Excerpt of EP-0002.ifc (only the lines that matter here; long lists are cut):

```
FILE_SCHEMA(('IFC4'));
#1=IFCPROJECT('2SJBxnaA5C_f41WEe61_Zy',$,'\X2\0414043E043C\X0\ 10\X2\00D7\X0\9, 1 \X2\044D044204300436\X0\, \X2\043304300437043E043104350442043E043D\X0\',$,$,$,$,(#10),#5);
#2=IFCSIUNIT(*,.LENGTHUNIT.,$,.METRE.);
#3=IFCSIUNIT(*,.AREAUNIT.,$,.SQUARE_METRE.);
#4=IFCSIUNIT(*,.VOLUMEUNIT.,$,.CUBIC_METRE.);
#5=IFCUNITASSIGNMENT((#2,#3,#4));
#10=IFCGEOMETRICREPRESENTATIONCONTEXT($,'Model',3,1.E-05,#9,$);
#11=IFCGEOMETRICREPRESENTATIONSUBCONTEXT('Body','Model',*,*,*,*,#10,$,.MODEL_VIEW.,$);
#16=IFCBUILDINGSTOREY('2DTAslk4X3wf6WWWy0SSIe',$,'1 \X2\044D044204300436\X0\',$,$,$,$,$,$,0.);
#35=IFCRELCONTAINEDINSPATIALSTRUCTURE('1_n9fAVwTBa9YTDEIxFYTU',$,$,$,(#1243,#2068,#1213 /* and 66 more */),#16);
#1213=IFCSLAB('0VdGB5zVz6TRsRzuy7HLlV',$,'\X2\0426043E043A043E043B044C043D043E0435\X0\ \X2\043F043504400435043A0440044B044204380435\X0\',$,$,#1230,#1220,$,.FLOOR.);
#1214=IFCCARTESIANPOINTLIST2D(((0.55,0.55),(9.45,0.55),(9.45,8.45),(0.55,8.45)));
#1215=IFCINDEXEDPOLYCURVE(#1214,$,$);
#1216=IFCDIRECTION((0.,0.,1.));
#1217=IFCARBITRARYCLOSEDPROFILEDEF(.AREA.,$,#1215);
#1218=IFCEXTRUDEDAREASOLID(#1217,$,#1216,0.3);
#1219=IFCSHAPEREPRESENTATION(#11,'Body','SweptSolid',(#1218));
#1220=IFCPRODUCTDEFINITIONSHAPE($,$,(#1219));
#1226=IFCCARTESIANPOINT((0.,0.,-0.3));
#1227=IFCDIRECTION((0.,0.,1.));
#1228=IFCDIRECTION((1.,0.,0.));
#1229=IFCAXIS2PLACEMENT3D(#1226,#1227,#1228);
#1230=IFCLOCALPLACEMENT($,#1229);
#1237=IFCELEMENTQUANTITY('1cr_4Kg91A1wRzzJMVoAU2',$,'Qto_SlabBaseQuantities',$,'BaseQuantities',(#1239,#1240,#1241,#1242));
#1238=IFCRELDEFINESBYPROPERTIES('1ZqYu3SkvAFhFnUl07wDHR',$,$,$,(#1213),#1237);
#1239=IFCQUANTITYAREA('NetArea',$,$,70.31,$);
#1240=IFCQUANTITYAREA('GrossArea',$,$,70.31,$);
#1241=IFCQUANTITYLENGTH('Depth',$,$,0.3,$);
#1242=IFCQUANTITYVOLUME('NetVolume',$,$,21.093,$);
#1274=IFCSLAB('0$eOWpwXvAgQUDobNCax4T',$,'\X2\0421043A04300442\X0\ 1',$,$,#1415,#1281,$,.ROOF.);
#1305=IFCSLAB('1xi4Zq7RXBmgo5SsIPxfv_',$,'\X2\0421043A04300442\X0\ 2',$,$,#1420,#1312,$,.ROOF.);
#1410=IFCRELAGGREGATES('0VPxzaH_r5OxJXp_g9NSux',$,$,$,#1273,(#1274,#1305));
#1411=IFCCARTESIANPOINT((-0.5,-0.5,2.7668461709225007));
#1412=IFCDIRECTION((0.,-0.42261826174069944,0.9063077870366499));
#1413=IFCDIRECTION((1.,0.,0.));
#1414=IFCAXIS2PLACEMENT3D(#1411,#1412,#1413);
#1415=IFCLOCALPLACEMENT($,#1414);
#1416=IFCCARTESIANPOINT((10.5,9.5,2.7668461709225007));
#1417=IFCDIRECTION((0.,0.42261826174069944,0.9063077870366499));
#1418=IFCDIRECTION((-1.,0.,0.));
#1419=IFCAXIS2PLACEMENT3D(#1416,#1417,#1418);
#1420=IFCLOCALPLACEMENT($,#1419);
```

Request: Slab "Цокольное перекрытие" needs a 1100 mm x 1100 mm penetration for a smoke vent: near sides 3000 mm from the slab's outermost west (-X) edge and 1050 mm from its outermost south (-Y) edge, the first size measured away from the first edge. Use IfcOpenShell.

```python
import numpy as np
import ifcopenshell
import ifcopenshell.api.feature
import ifcopenshell.api.geometry
import ifcopenshell.api.pset
import ifcopenshell.api.root
import ifcopenshell.geom
import ifcopenshell.util.element
import ifcopenshell.util.placement
import ifcopenshell.util.representation
import ifcopenshell.util.shape
import ifcopenshell.util.unit

model = ifcopenshell.open("EP-0002.ifc")
unit_scale = ifcopenshell.util.unit.calculate_unit_scale(model)
area_scale = ifcopenshell.util.unit.calculate_unit_scale(model, "AREAUNIT")
volume_scale = ifcopenshell.util.unit.calculate_unit_scale(model, "VOLUMEUNIT")
settings = ifcopenshell.geom.settings()


def volume(element):
    """Net volume in cubic metres, openings subtracted."""
    shape = ifcopenshell.geom.create_shape(settings, element)
    return ifcopenshell.util.shape.get_volume(shape.geometry)


slab = model.by_guid("0VdGB5zVz6TRsRzuy7HLlV")
before = volume(slab)

# Extent in the slab's own axes, in metres. The edges named are its -X and -Y sides.
slab_shape = ifcopenshell.geom.create_shape(settings, slab)
vertices = ifcopenshell.util.shape.get_vertices(slab_shape.geometry)
x_min, y_min, bottom = vertices.min(axis=0)
top = vertices[:, 2].max()

opening = ifcopenshell.api.root.create_entity(model, ifc_class="IfcOpeningElement", name="Smoke vent opening", predefined_type="OPENING")
context = ifcopenshell.util.representation.get_context(model, "Model", "Body", "MODEL_VIEW")
width, depth = 1.1, 1.1
outline = [(0.0, 0.0), (width, 0.0), (width, depth), (0.0, depth), (0.0, 0.0)]
# Overshoot both faces by 50 mm so the cut is clean.
shape = ifcopenshell.api.geometry.add_slab_representation(
    model, context=context, depth=top - bottom + 0.1, polyline=outline
)
ifcopenshell.api.geometry.assign_representation(model, product=opening, representation=shape)

matrix = ifcopenshell.util.placement.get_local_placement(slab.ObjectPlacement)
matrix[:, 3] = matrix @ np.append(np.array([x_min + 3, y_min + 1.05, bottom - 0.05]) / unit_scale, 1.0)
ifcopenshell.api.geometry.edit_object_placement(model, product=opening, matrix=matrix, is_si=False)
ifcopenshell.api.feature.add_feature(model, feature=opening, element=slab)

after = volume(slab)

# Update the slab's stored quantities.
qto = model.by_id(ifcopenshell.util.element.get_pset(slab, "Qto_SlabBaseQuantities", should_inherit=False)["id"])
ifcopenshell.api.pset.edit_qto(model, qto=qto, properties={
    "NetArea": after / (top - bottom) / area_scale,
    "NetVolume": after / volume_scale,
})

print(f"slab volume {before:.3f} -> {after:.3f} m3")

model.write("EP-0002_edited.ifc")
```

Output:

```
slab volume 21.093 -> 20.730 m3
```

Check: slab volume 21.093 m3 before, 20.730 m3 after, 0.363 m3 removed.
